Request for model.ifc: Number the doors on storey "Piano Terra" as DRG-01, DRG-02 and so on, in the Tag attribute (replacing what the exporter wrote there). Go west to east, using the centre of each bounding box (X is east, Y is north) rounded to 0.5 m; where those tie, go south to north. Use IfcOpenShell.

First a look at what the model holds.

```python
import ifcopenshell
import ifcopenshell.util.element
import ifcopenshell.util.placement

model = ifcopenshell.open("model.ifc")
print(model.schema)
storey = next(s for s in model.by_type("IfcBuildingStorey") if s.Name == "Piano Terra")
doors = [e for e in ifcopenshell.util.element.get_decomposition(storey) if e.is_a("IfcDoor")]
for e in sorted(doors, key=lambda e: e.id()):
    origin = ifcopenshell.util.placement.get_local_placement(e.ObjectPlacement)[:3, 3]
    print(e.id(), e.Tag, e.Name, origin.round(2) + 0.0, sep=" | ")
```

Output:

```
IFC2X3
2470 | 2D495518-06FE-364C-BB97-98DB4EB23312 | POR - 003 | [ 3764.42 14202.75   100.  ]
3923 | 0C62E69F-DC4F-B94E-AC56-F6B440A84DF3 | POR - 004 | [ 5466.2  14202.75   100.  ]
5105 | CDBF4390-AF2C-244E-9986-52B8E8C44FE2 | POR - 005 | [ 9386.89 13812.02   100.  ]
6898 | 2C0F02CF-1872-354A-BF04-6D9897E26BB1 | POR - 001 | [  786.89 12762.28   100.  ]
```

```python
import ifcopenshell
import ifcopenshell.geom
import ifcopenshell.util.element
import ifcopenshell.util.shape

model = ifcopenshell.open("model.ifc")
settings = ifcopenshell.geom.settings()
settings.set("use-world-coords", True)


def centre(element):
    shape = ifcopenshell.geom.create_shape(settings, element)
    return ifcopenshell.util.shape.get_bbox_centroid(shape.geometry)


storey = next(s for s in model.by_type("IfcBuildingStorey") if s.Name == "Piano Terra")
doors = [e for e in ifcopenshell.util.element.get_decomposition(storey) if e.is_a("IfcDoor")]

# Insertion points can sit at a corner or the storey origin, so sort by the geometry (in metres).
centres = {e: centre(e) for e in doors}
doors.sort(key=lambda e: (round(centres[e][0] / 0.5), centres[e][1]))

for i, e in enumerate(doors, start=1):
    number = f"DRG-{i:02d}"
    e.Tag = number
    print(e.id(), number)

model.write("model_rev.ifc")
```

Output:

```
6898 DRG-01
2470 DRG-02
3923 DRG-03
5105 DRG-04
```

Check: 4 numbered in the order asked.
